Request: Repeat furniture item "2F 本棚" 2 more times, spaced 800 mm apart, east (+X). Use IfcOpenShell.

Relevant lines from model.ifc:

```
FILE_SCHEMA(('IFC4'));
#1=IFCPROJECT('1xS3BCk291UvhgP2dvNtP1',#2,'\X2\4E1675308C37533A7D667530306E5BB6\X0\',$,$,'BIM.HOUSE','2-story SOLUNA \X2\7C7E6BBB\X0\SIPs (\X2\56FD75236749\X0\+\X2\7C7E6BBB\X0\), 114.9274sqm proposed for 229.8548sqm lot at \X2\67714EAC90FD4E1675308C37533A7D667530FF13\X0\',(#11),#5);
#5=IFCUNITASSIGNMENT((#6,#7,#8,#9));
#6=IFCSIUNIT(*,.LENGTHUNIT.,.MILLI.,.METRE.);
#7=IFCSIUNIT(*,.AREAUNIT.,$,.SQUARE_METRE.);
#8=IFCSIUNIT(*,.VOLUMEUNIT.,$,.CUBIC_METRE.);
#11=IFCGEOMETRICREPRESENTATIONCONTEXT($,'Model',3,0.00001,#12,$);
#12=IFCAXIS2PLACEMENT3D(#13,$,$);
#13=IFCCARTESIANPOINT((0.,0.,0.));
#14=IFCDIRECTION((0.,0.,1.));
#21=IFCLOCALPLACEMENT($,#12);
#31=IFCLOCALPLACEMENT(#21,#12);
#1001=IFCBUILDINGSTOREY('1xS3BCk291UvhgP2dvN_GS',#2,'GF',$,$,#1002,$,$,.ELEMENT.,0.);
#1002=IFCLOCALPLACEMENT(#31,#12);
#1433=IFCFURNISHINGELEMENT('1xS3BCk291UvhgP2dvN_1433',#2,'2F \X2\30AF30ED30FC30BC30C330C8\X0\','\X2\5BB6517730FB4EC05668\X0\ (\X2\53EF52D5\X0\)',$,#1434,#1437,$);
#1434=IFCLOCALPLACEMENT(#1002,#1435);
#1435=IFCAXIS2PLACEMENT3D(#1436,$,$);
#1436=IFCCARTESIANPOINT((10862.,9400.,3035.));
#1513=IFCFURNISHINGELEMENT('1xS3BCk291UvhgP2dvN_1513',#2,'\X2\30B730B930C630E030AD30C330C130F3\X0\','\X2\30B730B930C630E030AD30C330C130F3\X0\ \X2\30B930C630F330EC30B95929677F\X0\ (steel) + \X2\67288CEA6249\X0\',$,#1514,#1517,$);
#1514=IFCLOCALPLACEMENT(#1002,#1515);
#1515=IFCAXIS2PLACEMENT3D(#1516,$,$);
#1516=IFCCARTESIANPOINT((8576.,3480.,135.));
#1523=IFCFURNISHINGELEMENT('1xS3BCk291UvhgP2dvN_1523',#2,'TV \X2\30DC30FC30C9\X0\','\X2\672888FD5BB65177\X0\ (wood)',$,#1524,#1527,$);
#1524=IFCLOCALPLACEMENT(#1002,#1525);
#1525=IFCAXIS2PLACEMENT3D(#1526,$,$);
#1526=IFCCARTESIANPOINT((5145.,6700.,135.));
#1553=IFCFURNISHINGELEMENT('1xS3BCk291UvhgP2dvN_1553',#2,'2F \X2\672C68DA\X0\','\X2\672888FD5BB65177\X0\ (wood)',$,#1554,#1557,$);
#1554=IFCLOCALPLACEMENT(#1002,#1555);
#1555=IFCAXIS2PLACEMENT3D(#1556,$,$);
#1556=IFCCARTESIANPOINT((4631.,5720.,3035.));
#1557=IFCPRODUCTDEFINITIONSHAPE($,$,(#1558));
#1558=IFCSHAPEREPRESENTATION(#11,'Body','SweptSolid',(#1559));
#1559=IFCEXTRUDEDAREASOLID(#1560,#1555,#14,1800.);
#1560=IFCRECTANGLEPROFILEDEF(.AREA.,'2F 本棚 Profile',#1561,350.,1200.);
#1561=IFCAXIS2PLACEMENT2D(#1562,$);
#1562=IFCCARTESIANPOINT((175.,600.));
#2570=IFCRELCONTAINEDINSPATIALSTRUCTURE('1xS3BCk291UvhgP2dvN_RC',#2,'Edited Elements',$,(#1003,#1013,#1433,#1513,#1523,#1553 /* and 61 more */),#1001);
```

```python
import numpy as np
import ifcopenshell
import ifcopenshell.api.geometry
import ifcopenshell.api.root
import ifcopenshell.util.element
import ifcopenshell.util.placement

model = ifcopenshell.open("model.ifc")


def reuse_history(source, copy):
    """copy_class also copies each property set's owner history, people and application; keep the originals."""
    for rel in copy.IsDefinedBy:
        if rel.is_a("IfcRelDefinesByProperties") and (history := rel.RelatingPropertyDefinition.OwnerHistory):
            rel.RelatingPropertyDefinition.OwnerHistory = source.OwnerHistory
            ifcopenshell.util.element.remove_deep2(model, history)


source = model.by_guid("1xS3BCk291UvhgP2dvN_1553")
base = ifcopenshell.util.placement.get_local_placement(source.ObjectPlacement)
step = np.array([1.0, 0.0, 0.0]) * 800.0

for i in range(1, 3):
    copy = ifcopenshell.api.root.copy_class(model, product=source)
    copy.Representation = ifcopenshell.util.element.copy_deep(
        model, source.Representation, exclude=["IfcGeometricRepresentationContext", "IfcRepresentationMap"]
    )
    reuse_history(source, copy)
    matrix = base.copy()
    matrix[:3, 3] += i * step
    print("added at", matrix[:3, 3].round(3) + 0.0)
    ifcopenshell.api.geometry.edit_object_placement(model, product=copy, matrix=matrix, is_si=False)

model.write("model_edited.ifc")
```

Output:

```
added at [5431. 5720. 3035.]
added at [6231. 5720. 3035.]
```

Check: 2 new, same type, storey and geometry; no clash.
